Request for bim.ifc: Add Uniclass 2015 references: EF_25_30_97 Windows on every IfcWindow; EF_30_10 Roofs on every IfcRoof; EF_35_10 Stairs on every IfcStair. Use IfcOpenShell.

First a look at what the model holds.

```python
import ifcopenshell

model = ifcopenshell.open("bim.ifc")
print(model.schema)
print("classifications:", [c.Name for c in model.by_type("IfcClassification")])
for ifc_class in ("IfcDoor", "IfcRoof", "IfcStair", "IfcWall", "IfcWindow"):
    print(ifc_class, len(model.by_type(ifc_class)))
```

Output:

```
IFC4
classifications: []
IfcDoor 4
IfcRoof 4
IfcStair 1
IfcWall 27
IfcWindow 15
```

```python
import ifcopenshell
import ifcopenshell.api.classification

model = ifcopenshell.open("bim.ifc")

system = ifcopenshell.api.classification.add_classification(model, classification="Uniclass 2015")

codes = {
    "IfcWindow": ("EF_25_30_97", "Windows"),
    "IfcRoof": ("EF_30_10", "Roofs"),
    "IfcStair": ("EF_35_10", "Stairs"),
}
for ifc_class, (code, name) in codes.items():
    products = model.by_type(ifc_class)
    ifcopenshell.api.classification.add_reference(
        model, products=products, classification=system, identification=code, name=name
    )
    print(code, len(products))

model.write("bim_rev.ifc")
```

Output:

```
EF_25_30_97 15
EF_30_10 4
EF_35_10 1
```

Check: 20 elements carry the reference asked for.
